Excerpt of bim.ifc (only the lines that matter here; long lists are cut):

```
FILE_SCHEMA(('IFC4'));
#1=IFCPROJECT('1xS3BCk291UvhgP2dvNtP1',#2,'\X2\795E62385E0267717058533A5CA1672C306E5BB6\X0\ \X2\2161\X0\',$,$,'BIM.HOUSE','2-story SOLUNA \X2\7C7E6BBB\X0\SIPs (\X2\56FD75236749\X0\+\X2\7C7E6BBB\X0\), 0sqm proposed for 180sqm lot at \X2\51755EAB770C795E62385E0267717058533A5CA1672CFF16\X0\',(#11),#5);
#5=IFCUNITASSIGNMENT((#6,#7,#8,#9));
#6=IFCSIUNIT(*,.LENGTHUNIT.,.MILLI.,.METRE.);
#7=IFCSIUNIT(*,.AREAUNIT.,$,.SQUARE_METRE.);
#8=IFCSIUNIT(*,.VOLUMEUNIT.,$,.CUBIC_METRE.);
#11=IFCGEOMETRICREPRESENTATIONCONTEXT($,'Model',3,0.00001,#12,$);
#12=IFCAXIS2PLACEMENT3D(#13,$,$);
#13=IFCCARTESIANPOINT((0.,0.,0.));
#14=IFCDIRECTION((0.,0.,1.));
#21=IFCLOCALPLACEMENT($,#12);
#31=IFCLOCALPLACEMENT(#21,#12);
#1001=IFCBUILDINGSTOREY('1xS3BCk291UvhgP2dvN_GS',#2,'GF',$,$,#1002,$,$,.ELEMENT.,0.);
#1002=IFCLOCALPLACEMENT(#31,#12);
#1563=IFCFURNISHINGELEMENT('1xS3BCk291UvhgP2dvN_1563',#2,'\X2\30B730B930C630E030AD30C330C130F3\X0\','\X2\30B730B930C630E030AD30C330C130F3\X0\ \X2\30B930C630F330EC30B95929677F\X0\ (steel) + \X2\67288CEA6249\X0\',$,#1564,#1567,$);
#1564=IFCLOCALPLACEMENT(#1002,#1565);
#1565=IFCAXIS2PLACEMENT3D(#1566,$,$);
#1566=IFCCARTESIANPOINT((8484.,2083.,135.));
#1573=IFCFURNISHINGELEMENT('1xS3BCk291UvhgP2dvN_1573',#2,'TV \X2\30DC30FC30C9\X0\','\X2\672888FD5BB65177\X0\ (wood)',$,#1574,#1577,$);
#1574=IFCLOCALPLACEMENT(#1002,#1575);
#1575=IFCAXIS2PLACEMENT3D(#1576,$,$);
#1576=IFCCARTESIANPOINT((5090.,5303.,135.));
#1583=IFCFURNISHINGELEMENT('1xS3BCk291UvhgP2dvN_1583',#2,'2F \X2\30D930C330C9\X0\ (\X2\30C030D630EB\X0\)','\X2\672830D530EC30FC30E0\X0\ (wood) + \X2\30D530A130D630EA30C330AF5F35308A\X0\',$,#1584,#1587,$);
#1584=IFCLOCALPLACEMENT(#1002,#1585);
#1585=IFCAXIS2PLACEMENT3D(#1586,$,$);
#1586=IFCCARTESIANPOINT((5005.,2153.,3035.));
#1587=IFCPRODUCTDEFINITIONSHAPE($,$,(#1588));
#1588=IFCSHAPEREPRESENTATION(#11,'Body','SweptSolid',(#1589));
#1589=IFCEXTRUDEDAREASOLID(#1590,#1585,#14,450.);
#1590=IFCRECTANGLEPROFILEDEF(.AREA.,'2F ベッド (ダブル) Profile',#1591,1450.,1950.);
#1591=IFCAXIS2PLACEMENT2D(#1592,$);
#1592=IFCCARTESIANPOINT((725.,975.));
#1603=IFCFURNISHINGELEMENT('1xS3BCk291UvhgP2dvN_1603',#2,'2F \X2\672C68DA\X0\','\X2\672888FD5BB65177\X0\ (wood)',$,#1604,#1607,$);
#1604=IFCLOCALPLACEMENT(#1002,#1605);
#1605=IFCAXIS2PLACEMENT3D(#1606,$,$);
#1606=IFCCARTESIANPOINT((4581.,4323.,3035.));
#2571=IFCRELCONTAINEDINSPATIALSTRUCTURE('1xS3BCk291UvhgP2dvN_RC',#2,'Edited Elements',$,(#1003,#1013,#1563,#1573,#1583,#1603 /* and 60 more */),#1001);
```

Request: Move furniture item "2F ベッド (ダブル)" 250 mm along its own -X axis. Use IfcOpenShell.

```python
import ifcopenshell
import ifcopenshell.api.geometry
import ifcopenshell.util.placement

model = ifcopenshell.open("bim.ifc")

item = model.by_guid("1xS3BCk291UvhgP2dvN_1583")
matrix = ifcopenshell.util.placement.get_local_placement(item.ObjectPlacement)
matrix[:3, 3] -= matrix[:3, 0] * 250.0
ifcopenshell.api.geometry.edit_object_placement(model, product=item, matrix=matrix, is_si=False)

print(ifcopenshell.util.placement.get_local_placement(item.ObjectPlacement).round(3) + 0.0)

model.write("bim_edited.ifc")
```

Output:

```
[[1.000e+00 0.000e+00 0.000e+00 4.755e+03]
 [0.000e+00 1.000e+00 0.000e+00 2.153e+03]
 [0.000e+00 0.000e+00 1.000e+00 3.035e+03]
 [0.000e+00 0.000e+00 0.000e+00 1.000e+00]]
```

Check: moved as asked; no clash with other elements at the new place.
